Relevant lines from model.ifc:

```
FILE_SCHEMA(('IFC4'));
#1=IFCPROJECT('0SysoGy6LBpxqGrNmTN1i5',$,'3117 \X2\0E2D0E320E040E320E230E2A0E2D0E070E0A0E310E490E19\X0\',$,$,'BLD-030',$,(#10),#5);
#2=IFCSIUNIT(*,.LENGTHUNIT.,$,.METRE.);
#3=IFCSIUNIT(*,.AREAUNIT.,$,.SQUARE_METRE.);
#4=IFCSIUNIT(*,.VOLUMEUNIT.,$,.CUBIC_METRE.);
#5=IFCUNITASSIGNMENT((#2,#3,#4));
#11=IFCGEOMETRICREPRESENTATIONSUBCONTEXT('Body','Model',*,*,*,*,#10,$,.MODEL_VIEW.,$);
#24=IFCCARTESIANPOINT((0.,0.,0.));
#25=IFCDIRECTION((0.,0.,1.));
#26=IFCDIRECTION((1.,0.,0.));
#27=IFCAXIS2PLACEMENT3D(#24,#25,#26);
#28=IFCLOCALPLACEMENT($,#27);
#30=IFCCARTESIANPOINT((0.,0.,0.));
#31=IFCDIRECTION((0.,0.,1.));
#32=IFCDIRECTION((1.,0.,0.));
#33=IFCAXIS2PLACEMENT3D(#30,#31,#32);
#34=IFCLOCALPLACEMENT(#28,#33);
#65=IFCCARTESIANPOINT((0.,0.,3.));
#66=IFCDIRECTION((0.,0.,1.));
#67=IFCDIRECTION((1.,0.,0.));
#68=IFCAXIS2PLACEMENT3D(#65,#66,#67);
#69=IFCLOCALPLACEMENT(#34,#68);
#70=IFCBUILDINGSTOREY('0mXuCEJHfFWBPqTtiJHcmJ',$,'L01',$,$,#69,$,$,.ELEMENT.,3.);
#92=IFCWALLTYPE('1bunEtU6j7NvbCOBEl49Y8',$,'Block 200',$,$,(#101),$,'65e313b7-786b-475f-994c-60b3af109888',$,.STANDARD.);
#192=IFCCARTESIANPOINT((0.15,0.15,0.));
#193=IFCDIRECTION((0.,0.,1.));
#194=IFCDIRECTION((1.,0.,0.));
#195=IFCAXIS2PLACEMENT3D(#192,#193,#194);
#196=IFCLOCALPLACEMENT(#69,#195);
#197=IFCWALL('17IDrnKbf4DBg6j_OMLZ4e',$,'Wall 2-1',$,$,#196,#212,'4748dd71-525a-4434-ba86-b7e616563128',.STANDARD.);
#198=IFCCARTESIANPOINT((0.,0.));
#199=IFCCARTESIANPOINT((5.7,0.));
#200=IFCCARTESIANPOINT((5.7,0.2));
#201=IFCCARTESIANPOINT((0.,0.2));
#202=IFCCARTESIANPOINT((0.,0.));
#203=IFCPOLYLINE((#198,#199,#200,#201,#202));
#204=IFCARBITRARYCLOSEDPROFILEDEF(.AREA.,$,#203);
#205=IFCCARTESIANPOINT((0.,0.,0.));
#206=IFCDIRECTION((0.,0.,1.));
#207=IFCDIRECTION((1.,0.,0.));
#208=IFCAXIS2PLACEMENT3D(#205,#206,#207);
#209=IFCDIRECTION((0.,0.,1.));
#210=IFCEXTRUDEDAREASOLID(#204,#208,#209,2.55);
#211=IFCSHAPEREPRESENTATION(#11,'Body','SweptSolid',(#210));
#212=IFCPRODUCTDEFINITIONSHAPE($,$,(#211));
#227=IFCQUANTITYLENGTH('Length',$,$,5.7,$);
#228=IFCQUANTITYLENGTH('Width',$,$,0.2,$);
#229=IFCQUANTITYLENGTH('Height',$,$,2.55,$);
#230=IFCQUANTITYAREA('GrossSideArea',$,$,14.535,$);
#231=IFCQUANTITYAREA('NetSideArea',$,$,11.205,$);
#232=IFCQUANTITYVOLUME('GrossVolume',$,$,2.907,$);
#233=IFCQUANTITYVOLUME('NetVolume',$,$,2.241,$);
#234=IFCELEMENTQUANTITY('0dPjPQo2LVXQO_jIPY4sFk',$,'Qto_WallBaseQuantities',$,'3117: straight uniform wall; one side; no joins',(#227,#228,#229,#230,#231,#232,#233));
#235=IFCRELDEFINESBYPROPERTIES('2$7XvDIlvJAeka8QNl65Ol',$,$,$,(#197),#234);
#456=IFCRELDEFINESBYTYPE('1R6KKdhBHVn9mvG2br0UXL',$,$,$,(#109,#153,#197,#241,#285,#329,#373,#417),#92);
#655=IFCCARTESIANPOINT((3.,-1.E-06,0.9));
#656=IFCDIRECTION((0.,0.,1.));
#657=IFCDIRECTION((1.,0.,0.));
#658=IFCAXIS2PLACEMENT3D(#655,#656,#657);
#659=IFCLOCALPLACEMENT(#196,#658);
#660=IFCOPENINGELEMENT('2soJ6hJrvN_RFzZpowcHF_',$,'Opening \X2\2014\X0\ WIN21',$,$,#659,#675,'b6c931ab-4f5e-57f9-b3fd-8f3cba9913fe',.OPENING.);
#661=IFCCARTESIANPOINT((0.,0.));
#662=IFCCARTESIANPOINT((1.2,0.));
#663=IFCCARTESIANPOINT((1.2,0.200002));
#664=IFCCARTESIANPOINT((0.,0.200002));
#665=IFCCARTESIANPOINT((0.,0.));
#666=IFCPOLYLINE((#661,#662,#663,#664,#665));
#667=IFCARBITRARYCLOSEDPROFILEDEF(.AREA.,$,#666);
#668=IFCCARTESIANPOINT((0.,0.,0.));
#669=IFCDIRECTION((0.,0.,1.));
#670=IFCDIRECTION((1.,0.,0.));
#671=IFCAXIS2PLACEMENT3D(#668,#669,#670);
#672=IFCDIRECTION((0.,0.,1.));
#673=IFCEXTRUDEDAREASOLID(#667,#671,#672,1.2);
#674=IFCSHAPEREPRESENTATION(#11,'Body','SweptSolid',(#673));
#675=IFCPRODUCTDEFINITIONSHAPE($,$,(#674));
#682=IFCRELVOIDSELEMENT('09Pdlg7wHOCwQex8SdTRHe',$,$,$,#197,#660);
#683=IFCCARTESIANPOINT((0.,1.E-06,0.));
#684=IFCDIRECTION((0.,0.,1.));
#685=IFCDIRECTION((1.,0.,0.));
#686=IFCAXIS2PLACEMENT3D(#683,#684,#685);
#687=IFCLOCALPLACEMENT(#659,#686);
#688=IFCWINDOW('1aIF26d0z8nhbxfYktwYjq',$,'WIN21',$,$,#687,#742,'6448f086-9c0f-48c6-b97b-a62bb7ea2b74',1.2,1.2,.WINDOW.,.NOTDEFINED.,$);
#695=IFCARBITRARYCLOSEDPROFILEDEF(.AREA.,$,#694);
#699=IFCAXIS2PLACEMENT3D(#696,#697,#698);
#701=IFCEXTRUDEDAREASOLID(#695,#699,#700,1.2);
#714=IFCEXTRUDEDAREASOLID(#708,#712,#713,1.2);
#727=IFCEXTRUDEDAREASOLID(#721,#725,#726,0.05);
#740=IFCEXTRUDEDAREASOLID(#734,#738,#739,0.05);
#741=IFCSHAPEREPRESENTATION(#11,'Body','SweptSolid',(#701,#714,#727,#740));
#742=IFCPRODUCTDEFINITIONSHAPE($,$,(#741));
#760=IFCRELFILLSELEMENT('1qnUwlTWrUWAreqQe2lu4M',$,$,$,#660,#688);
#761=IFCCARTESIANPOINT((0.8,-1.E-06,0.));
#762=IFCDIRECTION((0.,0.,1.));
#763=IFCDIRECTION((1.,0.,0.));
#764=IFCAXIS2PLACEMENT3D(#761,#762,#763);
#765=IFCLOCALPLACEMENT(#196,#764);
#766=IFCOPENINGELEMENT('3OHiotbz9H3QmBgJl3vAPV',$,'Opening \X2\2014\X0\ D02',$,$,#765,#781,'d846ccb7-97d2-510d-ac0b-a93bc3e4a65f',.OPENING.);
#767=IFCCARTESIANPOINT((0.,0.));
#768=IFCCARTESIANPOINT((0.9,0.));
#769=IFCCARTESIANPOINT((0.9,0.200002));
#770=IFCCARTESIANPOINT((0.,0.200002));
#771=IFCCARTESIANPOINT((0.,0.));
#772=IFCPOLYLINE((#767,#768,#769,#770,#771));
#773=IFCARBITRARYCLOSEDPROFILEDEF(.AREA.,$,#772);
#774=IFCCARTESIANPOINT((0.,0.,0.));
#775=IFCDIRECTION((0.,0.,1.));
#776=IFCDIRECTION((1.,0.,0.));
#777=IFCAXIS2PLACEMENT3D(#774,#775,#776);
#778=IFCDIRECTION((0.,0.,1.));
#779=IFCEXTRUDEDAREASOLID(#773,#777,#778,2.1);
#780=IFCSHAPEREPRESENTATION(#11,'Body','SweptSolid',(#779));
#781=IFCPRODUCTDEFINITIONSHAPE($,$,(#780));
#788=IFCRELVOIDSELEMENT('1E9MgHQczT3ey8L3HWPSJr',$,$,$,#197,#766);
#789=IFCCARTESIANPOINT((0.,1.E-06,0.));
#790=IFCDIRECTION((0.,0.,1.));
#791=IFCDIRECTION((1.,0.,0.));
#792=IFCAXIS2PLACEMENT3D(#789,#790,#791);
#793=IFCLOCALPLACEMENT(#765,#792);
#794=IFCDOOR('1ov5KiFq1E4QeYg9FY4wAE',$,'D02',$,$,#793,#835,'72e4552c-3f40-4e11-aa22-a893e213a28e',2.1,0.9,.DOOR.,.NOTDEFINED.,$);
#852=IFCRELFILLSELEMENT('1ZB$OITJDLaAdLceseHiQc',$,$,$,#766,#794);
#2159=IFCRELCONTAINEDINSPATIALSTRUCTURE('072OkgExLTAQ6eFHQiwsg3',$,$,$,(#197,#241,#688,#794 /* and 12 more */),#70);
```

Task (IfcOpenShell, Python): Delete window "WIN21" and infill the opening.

```python
import ifcopenshell
import ifcopenshell.api.feature
import ifcopenshell.api.pset
import ifcopenshell.api.root
import ifcopenshell.geom
import ifcopenshell.util.element
import ifcopenshell.util.shape
import ifcopenshell.util.unit

model = ifcopenshell.open("model.ifc")
area_scale = ifcopenshell.util.unit.calculate_unit_scale(model, "AREAUNIT")
volume_scale = ifcopenshell.util.unit.calculate_unit_scale(model, "VOLUMEUNIT")
settings = ifcopenshell.geom.settings()


def volume(element):
    """Net volume in cubic metres, openings subtracted."""
    shape = ifcopenshell.geom.create_shape(settings, element)
    return ifcopenshell.util.shape.get_volume(shape.geometry)


window = model.by_guid("1aIF26d0z8nhbxfYktwYjq")
opening = window.FillsVoids[0].RelatingOpeningElement
wall = opening.VoidsElements[0].RelatingBuildingElement
before = volume(wall)

ifcopenshell.api.root.remove_product(model, product=window)
ifcopenshell.api.feature.remove_feature(model, feature=opening)

after = volume(wall)
thickness = 0.2  # wall thickness in metres

# Update the wall's stored quantities.
qto = model.by_id(ifcopenshell.util.element.get_pset(wall, "Qto_WallBaseQuantities", should_inherit=False)["id"])
ifcopenshell.api.pset.edit_qto(model, qto=qto, properties={
    "NetSideArea": after / thickness / area_scale,
    "NetVolume": after / volume_scale,
})

print(f"wall volume {before:.3f} -> {after:.3f} m3")

model.write("model_updated.ifc")
```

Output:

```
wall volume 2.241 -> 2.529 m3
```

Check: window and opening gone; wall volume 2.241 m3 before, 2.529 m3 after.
